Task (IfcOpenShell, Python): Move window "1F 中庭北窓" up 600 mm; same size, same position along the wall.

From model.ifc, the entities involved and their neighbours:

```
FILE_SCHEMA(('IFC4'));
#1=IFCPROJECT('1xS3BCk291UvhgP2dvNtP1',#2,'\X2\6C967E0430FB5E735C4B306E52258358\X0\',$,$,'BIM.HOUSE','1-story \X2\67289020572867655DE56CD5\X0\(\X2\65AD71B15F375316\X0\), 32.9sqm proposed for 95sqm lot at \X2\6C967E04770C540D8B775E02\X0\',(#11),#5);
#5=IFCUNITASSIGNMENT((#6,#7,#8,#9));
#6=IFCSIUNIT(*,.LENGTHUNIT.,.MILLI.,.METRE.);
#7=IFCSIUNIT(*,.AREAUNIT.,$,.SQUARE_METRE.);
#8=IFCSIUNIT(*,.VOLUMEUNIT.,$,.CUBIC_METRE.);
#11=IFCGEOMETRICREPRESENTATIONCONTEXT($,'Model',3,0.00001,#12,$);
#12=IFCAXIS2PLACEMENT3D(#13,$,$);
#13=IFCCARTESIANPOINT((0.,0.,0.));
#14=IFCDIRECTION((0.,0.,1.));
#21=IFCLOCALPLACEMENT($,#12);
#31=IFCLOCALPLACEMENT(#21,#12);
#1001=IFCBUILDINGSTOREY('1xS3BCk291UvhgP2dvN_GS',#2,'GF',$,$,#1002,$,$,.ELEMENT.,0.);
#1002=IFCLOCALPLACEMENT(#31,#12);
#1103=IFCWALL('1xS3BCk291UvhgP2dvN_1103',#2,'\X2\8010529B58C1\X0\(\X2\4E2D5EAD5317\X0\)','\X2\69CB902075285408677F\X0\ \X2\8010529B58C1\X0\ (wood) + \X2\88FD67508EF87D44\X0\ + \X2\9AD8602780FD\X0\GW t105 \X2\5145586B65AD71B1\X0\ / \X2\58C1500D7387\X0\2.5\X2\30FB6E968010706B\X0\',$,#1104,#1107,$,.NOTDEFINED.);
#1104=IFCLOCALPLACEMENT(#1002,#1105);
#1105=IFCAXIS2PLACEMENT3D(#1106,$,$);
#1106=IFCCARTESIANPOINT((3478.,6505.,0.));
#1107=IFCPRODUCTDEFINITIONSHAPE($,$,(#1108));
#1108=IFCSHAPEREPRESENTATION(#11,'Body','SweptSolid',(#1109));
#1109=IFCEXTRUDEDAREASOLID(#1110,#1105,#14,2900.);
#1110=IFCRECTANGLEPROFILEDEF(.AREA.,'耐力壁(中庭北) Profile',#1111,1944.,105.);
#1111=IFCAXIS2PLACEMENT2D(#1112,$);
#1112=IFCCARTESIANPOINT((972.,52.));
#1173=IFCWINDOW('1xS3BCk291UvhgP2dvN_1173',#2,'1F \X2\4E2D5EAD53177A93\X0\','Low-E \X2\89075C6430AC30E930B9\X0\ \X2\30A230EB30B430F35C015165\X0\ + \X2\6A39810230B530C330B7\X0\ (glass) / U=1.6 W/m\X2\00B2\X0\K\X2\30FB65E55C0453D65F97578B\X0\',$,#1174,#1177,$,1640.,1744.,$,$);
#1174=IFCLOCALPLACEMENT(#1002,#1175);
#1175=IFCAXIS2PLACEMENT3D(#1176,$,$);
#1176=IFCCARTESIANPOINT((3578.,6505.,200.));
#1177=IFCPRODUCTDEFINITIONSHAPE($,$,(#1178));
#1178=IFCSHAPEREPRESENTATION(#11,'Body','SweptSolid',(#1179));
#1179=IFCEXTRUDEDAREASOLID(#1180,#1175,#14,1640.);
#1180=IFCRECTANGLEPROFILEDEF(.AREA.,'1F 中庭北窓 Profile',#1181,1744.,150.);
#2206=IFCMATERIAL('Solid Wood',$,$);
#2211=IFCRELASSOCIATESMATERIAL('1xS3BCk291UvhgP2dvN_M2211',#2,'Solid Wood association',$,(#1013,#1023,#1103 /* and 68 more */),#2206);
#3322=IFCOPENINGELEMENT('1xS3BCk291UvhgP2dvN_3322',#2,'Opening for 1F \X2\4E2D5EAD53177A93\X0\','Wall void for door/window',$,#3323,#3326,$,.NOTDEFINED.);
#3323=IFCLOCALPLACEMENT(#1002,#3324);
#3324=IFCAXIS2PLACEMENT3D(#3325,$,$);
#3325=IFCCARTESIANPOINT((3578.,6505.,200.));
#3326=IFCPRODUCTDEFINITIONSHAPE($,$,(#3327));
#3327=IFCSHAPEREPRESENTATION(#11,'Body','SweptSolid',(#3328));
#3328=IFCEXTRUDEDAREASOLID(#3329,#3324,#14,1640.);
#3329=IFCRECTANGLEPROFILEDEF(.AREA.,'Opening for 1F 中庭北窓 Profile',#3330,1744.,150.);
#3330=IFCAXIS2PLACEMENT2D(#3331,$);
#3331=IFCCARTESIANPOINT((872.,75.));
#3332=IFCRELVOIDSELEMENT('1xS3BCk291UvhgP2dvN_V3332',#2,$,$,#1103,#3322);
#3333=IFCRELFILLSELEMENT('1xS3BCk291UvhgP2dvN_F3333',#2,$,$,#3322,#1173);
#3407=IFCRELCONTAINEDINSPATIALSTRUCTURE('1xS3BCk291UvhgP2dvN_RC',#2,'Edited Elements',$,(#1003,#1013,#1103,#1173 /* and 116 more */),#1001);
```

```python
import numpy as np
import ifcopenshell
import ifcopenshell.api.geometry
import ifcopenshell.util.placement
import ifcopenshell.util.unit

model = ifcopenshell.open("model.ifc")
unit_scale = ifcopenshell.util.unit.calculate_unit_scale(model)

window = model.by_guid("1xS3BCk291UvhgP2dvN_1173")
opening = window.FillsVoids[0].RelatingOpeningElement
dz = 0.6 / unit_scale

shift = np.array([0.0, 0.0, dz])
# The window is not placed relative to its opening, so move both.
for product in (opening, window):
    matrix = ifcopenshell.util.placement.get_local_placement(product.ObjectPlacement)
    matrix[:3, 3] += shift
    ifcopenshell.api.geometry.edit_object_placement(model, product=product, matrix=matrix, is_si=False)

print(f"moved by {dz * unit_scale:+.3f} m")

model.write("model_rev.ifc")
```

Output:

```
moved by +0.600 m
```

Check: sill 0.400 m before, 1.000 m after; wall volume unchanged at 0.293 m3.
